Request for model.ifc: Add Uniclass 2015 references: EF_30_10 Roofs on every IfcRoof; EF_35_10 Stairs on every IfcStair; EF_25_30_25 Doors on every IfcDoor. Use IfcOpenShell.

First a look at what the model holds.

```python
import ifcopenshell

model = ifcopenshell.open("model.ifc")
print(model.schema)
print("classifications:", [c.Name for c in model.by_type("IfcClassification")])
for ifc_class in ("IfcDoor", "IfcRoof", "IfcStair", "IfcWall", "IfcWindow"):
    print(ifc_class, len(model.by_type(ifc_class)))
```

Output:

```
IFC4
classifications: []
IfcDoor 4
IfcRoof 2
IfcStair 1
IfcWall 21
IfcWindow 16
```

```python
import ifcopenshell
import ifcopenshell.api.classification

model = ifcopenshell.open("model.ifc")

system = ifcopenshell.api.classification.add_classification(model, classification="Uniclass 2015")

codes = {
    "IfcRoof": ("EF_30_10", "Roofs"),
    "IfcStair": ("EF_35_10", "Stairs"),
    "IfcDoor": ("EF_25_30_25", "Doors"),
}
for ifc_class, (code, name) in codes.items():
    products = model.by_type(ifc_class)
    ifcopenshell.api.classification.add_reference(
        model, products=products, classification=system, identification=code, name=name
    )
    print(code, len(products))

model.write("model-out.ifc")
```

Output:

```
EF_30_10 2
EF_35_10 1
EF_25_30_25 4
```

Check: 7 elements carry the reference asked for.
